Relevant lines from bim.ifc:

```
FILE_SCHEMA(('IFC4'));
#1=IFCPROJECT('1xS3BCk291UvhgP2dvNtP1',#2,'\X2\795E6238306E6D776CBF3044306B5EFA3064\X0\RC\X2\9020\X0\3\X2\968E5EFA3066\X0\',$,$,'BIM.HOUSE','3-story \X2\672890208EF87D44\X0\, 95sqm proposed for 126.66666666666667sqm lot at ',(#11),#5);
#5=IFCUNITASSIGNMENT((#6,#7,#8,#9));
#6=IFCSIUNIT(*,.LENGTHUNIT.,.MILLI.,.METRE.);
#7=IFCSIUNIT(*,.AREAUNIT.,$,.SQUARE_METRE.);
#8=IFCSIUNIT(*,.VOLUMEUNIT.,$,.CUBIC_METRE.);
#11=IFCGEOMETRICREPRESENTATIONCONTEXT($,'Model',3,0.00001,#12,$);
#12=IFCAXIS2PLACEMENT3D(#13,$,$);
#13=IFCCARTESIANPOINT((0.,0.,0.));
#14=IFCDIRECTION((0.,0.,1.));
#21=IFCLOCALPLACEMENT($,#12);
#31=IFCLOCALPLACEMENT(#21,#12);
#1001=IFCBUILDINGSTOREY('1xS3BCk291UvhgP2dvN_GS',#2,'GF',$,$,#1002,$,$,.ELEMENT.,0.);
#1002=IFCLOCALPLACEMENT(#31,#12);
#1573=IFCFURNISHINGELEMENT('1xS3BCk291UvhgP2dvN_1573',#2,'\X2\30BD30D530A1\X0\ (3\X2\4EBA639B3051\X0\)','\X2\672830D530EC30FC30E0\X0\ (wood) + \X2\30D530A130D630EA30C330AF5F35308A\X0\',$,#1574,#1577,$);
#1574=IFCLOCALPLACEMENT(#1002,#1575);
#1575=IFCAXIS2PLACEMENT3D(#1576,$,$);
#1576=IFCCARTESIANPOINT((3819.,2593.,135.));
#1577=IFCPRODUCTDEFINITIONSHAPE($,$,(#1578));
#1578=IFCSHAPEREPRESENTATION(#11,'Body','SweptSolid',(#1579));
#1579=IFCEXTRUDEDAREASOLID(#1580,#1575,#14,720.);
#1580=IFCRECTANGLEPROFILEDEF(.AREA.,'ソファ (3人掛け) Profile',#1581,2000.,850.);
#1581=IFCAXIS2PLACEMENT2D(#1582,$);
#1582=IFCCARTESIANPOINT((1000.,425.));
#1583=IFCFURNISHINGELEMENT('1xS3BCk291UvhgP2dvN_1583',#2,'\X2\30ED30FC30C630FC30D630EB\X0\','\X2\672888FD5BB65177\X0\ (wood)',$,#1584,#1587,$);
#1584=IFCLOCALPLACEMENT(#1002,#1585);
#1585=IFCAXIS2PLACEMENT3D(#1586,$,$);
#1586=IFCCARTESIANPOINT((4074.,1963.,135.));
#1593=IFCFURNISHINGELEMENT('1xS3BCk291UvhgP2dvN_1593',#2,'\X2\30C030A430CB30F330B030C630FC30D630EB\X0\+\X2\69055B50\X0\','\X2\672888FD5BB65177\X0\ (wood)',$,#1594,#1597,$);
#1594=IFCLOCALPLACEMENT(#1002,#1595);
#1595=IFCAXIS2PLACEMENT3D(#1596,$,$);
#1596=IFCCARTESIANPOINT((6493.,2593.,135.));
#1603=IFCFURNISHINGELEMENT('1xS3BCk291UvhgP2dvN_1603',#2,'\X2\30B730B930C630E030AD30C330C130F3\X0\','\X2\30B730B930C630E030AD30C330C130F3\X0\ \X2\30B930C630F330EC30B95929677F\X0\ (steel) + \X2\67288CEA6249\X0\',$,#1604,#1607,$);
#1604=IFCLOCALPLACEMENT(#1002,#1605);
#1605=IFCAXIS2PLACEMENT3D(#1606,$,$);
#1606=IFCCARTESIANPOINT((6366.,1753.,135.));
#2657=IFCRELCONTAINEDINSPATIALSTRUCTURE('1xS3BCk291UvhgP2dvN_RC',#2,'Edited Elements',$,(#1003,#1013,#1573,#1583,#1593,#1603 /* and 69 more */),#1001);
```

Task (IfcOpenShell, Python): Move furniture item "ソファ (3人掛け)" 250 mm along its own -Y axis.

```python
import ifcopenshell
import ifcopenshell.api.geometry
import ifcopenshell.util.placement
import ifcopenshell.util.unit

model = ifcopenshell.open("bim.ifc")
unit_scale = ifcopenshell.util.unit.calculate_unit_scale(model)

item = model.by_guid("1xS3BCk291UvhgP2dvN_1573")
matrix = ifcopenshell.util.placement.get_local_placement(item.ObjectPlacement)
matrix[:3, 3] -= matrix[:3, 1] * 0.25 / unit_scale
ifcopenshell.api.geometry.edit_object_placement(model, product=item, matrix=matrix, is_si=False)

print(ifcopenshell.util.placement.get_local_placement(item.ObjectPlacement).round(3) + 0.0)

model.write("bim_rev.ifc")
```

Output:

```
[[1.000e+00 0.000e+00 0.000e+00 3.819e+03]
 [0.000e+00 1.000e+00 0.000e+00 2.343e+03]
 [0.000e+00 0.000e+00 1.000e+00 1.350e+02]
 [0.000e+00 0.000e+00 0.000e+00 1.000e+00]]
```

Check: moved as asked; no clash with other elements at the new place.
